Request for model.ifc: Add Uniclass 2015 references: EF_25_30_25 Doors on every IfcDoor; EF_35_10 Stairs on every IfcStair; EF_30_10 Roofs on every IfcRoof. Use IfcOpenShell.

First a look at what the model holds.

```python
import ifcopenshell

model = ifcopenshell.open("model.ifc")
print(model.schema)
print("classifications:", [c.Name for c in model.by_type("IfcClassification")])
for ifc_class in ("IfcDoor", "IfcRoof", "IfcStair", "IfcWall", "IfcWindow"):
    print(ifc_class, len(model.by_type(ifc_class)))
```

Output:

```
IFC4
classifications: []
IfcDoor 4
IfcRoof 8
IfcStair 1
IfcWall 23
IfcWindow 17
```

```python
import ifcopenshell
import ifcopenshell.api.classification

model = ifcopenshell.open("model.ifc")

system = ifcopenshell.api.classification.add_classification(model, classification="Uniclass 2015")

codes = {
    "IfcDoor": ("EF_25_30_25", "Doors"),
    "IfcStair": ("EF_35_10", "Stairs"),
    "IfcRoof": ("EF_30_10", "Roofs"),
}
for ifc_class, (code, name) in codes.items():
    products = model.by_type(ifc_class)
    ifcopenshell.api.classification.add_reference(
        model, products=products, classification=system, identification=code, name=name
    )
    print(code, len(products))

model.write("model_v2.ifc")
```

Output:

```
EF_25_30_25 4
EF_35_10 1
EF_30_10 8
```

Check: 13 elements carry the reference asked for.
